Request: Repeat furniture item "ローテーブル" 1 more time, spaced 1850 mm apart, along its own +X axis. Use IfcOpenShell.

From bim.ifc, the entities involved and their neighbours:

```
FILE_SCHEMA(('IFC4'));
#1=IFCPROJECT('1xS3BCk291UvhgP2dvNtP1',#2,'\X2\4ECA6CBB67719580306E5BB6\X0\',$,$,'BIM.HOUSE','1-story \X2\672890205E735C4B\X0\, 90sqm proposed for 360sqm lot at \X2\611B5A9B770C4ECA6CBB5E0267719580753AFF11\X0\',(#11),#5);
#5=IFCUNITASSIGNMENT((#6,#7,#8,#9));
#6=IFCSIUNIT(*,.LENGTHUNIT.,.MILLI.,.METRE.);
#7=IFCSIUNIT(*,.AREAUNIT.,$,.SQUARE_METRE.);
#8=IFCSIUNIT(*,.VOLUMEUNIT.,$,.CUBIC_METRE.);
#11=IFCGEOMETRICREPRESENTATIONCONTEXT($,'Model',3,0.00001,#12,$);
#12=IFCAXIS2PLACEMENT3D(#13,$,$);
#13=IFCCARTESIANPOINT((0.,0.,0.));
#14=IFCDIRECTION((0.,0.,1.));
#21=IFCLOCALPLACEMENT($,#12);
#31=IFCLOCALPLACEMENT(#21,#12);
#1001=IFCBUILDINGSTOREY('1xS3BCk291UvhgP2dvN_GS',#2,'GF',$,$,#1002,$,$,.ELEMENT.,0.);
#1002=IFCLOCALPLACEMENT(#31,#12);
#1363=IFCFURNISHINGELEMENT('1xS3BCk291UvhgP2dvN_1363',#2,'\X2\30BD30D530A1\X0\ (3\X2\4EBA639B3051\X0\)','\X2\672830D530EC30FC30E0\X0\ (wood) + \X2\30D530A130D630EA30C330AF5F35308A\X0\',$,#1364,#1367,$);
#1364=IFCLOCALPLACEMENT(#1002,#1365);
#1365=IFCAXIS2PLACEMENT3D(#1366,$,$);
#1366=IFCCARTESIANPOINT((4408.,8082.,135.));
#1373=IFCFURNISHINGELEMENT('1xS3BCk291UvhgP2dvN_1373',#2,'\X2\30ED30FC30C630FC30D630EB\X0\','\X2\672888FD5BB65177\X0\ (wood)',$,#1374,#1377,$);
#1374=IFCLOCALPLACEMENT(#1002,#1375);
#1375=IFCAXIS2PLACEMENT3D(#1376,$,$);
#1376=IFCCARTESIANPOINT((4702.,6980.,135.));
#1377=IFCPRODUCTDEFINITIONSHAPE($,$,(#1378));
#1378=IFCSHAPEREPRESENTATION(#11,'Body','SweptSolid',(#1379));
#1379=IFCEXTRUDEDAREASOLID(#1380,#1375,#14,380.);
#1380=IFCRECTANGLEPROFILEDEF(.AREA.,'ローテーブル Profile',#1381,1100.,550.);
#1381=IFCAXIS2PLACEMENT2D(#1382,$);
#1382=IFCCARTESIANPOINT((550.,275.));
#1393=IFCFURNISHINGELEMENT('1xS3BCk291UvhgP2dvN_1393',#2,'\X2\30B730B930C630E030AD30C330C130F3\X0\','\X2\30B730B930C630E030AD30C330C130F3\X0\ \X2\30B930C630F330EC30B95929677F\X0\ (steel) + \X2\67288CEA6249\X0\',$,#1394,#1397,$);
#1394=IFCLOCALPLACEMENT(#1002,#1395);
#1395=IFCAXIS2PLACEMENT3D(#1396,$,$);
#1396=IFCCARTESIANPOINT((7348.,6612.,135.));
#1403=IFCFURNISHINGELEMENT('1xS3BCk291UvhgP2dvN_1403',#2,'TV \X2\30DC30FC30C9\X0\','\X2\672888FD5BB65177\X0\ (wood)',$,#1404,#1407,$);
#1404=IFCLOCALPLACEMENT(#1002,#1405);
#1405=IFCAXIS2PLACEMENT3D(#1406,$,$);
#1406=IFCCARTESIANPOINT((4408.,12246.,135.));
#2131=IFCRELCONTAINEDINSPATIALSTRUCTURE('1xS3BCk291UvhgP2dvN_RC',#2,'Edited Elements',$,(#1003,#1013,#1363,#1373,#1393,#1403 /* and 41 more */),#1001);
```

```python
import ifcopenshell
import ifcopenshell.api.geometry
import ifcopenshell.api.root
import ifcopenshell.util.element
import ifcopenshell.util.placement

model = ifcopenshell.open("bim.ifc")


def reuse_history(source, copy):
    """copy_class also copies each property set's owner history, people and application; keep the originals."""
    for rel in copy.IsDefinedBy:
        if rel.is_a("IfcRelDefinesByProperties") and (history := rel.RelatingPropertyDefinition.OwnerHistory):
            rel.RelatingPropertyDefinition.OwnerHistory = source.OwnerHistory
            ifcopenshell.util.element.remove_deep2(model, history)


source = model.by_guid("1xS3BCk291UvhgP2dvN_1373")
base = ifcopenshell.util.placement.get_local_placement(source.ObjectPlacement)
step = base[:3, 0] * 1850.0

for i in range(1, 2):
    copy = ifcopenshell.api.root.copy_class(model, product=source)
    copy.Representation = ifcopenshell.util.element.copy_deep(
        model, source.Representation, exclude=["IfcGeometricRepresentationContext", "IfcRepresentationMap"]
    )
    reuse_history(source, copy)
    matrix = base.copy()
    matrix[:3, 3] += i * step
    print("added at", matrix[:3, 3].round(3) + 0.0)
    ifcopenshell.api.geometry.edit_object_placement(model, product=copy, matrix=matrix, is_si=False)

model.write("bim_v2.ifc")
```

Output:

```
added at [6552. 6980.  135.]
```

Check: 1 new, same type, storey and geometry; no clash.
